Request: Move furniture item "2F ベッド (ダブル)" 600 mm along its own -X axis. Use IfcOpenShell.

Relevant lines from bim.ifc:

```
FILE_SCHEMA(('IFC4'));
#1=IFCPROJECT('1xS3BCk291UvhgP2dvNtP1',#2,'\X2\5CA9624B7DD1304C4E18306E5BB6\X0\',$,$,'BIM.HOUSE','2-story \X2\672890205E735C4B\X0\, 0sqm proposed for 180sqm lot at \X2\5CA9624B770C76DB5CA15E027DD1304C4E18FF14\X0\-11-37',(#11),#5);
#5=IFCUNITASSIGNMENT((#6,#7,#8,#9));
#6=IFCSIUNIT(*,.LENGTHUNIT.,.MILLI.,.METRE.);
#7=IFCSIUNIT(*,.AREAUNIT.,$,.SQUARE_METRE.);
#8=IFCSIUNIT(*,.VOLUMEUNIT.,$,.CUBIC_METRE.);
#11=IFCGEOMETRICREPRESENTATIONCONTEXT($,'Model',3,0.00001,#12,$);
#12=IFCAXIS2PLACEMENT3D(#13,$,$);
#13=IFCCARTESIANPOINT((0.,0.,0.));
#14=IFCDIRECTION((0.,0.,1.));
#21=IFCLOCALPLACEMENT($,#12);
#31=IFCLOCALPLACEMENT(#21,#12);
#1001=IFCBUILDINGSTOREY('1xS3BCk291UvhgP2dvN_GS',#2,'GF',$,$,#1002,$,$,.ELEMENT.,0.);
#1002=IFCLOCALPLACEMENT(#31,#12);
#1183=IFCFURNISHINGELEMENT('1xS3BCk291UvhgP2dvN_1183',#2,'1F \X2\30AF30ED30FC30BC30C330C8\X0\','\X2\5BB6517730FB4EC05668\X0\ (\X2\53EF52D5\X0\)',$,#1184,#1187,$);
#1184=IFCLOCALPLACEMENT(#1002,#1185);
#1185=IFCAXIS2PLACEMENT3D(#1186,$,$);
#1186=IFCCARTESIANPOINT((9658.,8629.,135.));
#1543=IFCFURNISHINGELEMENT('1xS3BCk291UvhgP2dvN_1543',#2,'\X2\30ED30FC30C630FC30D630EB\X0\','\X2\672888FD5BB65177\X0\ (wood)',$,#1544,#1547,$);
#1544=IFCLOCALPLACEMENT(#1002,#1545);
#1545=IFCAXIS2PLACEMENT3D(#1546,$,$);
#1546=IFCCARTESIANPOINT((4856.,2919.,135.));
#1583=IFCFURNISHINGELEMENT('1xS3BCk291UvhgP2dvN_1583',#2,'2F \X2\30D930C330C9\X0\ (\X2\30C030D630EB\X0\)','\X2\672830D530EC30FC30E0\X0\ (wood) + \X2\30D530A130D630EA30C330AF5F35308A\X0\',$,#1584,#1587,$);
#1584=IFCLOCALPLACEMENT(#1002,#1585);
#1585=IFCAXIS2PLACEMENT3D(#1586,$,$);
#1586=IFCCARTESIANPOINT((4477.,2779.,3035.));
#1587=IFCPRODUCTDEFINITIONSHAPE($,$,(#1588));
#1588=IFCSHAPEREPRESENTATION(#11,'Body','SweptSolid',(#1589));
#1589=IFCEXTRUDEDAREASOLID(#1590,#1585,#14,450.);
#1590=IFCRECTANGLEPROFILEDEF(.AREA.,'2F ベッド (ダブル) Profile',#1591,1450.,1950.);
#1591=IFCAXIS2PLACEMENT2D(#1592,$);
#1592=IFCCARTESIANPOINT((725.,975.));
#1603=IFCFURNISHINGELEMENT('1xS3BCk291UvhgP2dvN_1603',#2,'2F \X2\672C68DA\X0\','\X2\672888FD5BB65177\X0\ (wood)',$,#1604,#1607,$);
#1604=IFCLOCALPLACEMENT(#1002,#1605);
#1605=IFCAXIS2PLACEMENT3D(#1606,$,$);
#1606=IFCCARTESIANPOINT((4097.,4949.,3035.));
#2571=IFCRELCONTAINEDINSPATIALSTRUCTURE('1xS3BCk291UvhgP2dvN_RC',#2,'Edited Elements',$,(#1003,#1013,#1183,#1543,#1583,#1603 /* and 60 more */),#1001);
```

```python
import ifcopenshell
import ifcopenshell.api.geometry
import ifcopenshell.util.placement

model = ifcopenshell.open("bim.ifc")

item = model.by_guid("1xS3BCk291UvhgP2dvN_1583")
matrix = ifcopenshell.util.placement.get_local_placement(item.ObjectPlacement)
matrix[:3, 3] -= matrix[:3, 0] * 600.0
ifcopenshell.api.geometry.edit_object_placement(model, product=item, matrix=matrix, is_si=False)

print(ifcopenshell.util.placement.get_local_placement(item.ObjectPlacement).round(3) + 0.0)

model.write("bim_rev.ifc")
```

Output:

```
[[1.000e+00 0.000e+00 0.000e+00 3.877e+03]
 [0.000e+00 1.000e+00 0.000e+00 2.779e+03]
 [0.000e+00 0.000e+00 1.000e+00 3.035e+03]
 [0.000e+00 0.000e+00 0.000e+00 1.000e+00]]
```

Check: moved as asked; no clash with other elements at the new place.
